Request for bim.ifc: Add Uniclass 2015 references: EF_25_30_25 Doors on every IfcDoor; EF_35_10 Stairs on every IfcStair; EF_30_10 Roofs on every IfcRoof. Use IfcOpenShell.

First a look at what the model holds.

```python
import ifcopenshell

model = ifcopenshell.open("bim.ifc")
print(model.schema)
print("classifications:", [c.Name for c in model.by_type("IfcClassification")])
for ifc_class in ("IfcDoor", "IfcRoof", "IfcStair", "IfcWall", "IfcWindow"):
    print(ifc_class, len(model.by_type(ifc_class)))
```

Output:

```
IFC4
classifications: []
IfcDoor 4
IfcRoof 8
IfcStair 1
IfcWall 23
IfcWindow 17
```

```python
import ifcopenshell
import ifcopenshell.api.classification

model = ifcopenshell.open("bim.ifc")

system = ifcopenshell.api.classification.add_classification(model, classification="Uniclass 2015")

codes = {
    "IfcDoor": ("EF_25_30_25", "Doors"),
    "IfcStair": ("EF_35_10", "Stairs"),
    "IfcRoof": ("EF_30_10", "Roofs"),
}
for ifc_class, (code, name) in codes.items():
    products = model.by_type(ifc_class)
    ifcopenshell.api.classification.add_reference(
        model, products=products, classification=system, identification=code, name=name
    )
    print(code, len(products))

model.write("bim_v2.ifc")
```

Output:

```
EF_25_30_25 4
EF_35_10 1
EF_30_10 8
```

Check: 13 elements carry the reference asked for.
